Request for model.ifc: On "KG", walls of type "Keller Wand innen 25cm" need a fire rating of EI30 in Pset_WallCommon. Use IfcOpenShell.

First a look at what the model holds.

```python
import ifcopenshell
import ifcopenshell.util.element

model = ifcopenshell.open("model.ifc")
print(model.schema)
storey = next(s for s in model.by_type("IfcBuildingStorey") if s.Name == "KG")
walls = [e for e in ifcopenshell.util.element.get_decomposition(storey) if e.is_a("IfcWall")]
seen = {}
for e in walls:
    element_type = ifcopenshell.util.element.get_type(e)
    key = (element_type.Name if element_type != e and element_type else None, ifcopenshell.util.element.get_pset(e, "Pset_WallCommon", "FireRating"))
    seen[key] = seen.get(key, 0) + 1
for (name, value), count in sorted(seen.items(), key=str):
    print(count, "x", name, "|", value)
```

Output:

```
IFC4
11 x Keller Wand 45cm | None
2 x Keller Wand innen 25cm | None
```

```python
import ifcopenshell
import ifcopenshell.api.pset
import ifcopenshell.util.element

model = ifcopenshell.open("model.ifc")

storey = next(s for s in model.by_type("IfcBuildingStorey") if s.Name == "KG")
walls = [e for e in ifcopenshell.util.element.get_decomposition(storey) if e.is_a("IfcWall")]

count = 0
for e in walls:
    element_type = ifcopenshell.util.element.get_type(e)
    if element_type in (None, e) or element_type.Name != "Keller Wand innen 25cm":
        continue
    # add_pset returns the element's existing set when there is one.
    pset = ifcopenshell.api.pset.add_pset(model, product=e, name="Pset_WallCommon")
    ifcopenshell.api.pset.edit_pset(model, pset=pset, properties={"FireRating": "EI30"})
    count += 1

print(count, "walls updated")

model.write("model_rev.ifc")
```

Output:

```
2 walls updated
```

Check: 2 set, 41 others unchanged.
